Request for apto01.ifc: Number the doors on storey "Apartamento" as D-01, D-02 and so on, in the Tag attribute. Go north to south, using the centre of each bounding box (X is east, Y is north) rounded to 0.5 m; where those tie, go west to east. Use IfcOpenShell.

First a look at what the model holds.

```python
import ifcopenshell
import ifcopenshell.util.element
import ifcopenshell.util.placement

model = ifcopenshell.open("apto01.ifc")
print(model.schema)
storey = next(s for s in model.by_type("IfcBuildingStorey") if s.Name == "Apartamento")
doors = [e for e in ifcopenshell.util.element.get_decomposition(storey) if e.is_a("IfcDoor")]
for e in sorted(doors, key=lambda e: e.id()):
    origin = ifcopenshell.util.placement.get_local_placement(e.ObjectPlacement)[:3, 3]
    print(e.id(), e.Tag, e.Name, origin.round(2) + 0.0, sep=" | ")
```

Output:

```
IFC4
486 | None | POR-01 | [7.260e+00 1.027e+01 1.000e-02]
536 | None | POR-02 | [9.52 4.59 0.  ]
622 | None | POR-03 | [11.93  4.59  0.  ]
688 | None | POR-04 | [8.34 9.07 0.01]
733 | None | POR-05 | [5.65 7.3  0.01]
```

```python
import ifcopenshell
import ifcopenshell.geom
import ifcopenshell.util.element
import ifcopenshell.util.shape

model = ifcopenshell.open("apto01.ifc")
settings = ifcopenshell.geom.settings()
settings.set("use-world-coords", True)


def centre(element):
    shape = ifcopenshell.geom.create_shape(settings, element)
    return ifcopenshell.util.shape.get_bbox_centroid(shape.geometry)


storey = next(s for s in model.by_type("IfcBuildingStorey") if s.Name == "Apartamento")
doors = [e for e in ifcopenshell.util.element.get_decomposition(storey) if e.is_a("IfcDoor")]

# Insertion points can sit at a corner or the storey origin, so sort by the geometry (in metres).
centres = {e: centre(e) for e in doors}
doors.sort(key=lambda e: (-round(centres[e][1] / 0.5), centres[e][0]))

for i, e in enumerate(doors, start=1):
    number = f"D-{i:02d}"
    e.Tag = number
    print(e.id(), number)

model.write("apto01_edited.ifc")
```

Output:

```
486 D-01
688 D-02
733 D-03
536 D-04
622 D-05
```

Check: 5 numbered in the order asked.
